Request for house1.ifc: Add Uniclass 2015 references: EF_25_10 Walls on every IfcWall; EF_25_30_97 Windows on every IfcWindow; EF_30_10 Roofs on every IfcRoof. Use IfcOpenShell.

First a look at what the model holds.

```python
import ifcopenshell

model = ifcopenshell.open("house1.ifc")
print(model.schema)
print("classifications:", [c.Name for c in model.by_type("IfcClassification")])
for ifc_class in ("IfcDoor", "IfcRoof", "IfcStair", "IfcWall", "IfcWindow"):
    print(ifc_class, len(model.by_type(ifc_class)))
```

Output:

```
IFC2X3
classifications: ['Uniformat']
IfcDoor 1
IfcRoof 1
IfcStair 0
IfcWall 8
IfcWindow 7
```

```python
import ifcopenshell
import ifcopenshell.api.classification

model = ifcopenshell.open("house1.ifc")

# IFC2X3 requires Source and Edition and has no link from the project to the system.
system = model.create_entity("IfcClassification", Source="NBS", Edition="2015", Name="Uniclass 2015")

codes = {
    "IfcWall": ("EF_25_10", "Walls"),
    "IfcWindow": ("EF_25_30_97", "Windows"),
    "IfcRoof": ("EF_30_10", "Roofs"),
}
for ifc_class, (code, name) in codes.items():
    products = model.by_type(ifc_class)
    ifcopenshell.api.classification.add_reference(
        model, products=products, classification=system, identification=code, name=name
    )
    print(code, len(products))

model.write("house1_rev.ifc")
```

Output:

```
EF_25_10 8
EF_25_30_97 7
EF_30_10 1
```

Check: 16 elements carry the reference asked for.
